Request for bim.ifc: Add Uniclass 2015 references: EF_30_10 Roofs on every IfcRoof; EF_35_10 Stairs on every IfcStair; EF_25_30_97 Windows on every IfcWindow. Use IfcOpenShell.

First a look at what the model holds.

```python
import ifcopenshell

model = ifcopenshell.open("bim.ifc")
print(model.schema)
print("classifications:", [c.Name for c in model.by_type("IfcClassification")])
for ifc_class in ("IfcDoor", "IfcRoof", "IfcStair", "IfcWall", "IfcWindow"):
    print(ifc_class, len(model.by_type(ifc_class)))
```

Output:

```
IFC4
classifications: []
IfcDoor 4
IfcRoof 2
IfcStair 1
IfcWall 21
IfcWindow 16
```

```python
import ifcopenshell
import ifcopenshell.api.classification

model = ifcopenshell.open("bim.ifc")

system = ifcopenshell.api.classification.add_classification(model, classification="Uniclass 2015")

codes = {
    "IfcRoof": ("EF_30_10", "Roofs"),
    "IfcStair": ("EF_35_10", "Stairs"),
    "IfcWindow": ("EF_25_30_97", "Windows"),
}
for ifc_class, (code, name) in codes.items():
    products = model.by_type(ifc_class)
    ifcopenshell.api.classification.add_reference(
        model, products=products, classification=system, identification=code, name=name
    )
    print(code, len(products))

model.write("bim_v2.ifc")
```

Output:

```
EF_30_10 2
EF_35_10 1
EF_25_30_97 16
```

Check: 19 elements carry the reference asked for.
